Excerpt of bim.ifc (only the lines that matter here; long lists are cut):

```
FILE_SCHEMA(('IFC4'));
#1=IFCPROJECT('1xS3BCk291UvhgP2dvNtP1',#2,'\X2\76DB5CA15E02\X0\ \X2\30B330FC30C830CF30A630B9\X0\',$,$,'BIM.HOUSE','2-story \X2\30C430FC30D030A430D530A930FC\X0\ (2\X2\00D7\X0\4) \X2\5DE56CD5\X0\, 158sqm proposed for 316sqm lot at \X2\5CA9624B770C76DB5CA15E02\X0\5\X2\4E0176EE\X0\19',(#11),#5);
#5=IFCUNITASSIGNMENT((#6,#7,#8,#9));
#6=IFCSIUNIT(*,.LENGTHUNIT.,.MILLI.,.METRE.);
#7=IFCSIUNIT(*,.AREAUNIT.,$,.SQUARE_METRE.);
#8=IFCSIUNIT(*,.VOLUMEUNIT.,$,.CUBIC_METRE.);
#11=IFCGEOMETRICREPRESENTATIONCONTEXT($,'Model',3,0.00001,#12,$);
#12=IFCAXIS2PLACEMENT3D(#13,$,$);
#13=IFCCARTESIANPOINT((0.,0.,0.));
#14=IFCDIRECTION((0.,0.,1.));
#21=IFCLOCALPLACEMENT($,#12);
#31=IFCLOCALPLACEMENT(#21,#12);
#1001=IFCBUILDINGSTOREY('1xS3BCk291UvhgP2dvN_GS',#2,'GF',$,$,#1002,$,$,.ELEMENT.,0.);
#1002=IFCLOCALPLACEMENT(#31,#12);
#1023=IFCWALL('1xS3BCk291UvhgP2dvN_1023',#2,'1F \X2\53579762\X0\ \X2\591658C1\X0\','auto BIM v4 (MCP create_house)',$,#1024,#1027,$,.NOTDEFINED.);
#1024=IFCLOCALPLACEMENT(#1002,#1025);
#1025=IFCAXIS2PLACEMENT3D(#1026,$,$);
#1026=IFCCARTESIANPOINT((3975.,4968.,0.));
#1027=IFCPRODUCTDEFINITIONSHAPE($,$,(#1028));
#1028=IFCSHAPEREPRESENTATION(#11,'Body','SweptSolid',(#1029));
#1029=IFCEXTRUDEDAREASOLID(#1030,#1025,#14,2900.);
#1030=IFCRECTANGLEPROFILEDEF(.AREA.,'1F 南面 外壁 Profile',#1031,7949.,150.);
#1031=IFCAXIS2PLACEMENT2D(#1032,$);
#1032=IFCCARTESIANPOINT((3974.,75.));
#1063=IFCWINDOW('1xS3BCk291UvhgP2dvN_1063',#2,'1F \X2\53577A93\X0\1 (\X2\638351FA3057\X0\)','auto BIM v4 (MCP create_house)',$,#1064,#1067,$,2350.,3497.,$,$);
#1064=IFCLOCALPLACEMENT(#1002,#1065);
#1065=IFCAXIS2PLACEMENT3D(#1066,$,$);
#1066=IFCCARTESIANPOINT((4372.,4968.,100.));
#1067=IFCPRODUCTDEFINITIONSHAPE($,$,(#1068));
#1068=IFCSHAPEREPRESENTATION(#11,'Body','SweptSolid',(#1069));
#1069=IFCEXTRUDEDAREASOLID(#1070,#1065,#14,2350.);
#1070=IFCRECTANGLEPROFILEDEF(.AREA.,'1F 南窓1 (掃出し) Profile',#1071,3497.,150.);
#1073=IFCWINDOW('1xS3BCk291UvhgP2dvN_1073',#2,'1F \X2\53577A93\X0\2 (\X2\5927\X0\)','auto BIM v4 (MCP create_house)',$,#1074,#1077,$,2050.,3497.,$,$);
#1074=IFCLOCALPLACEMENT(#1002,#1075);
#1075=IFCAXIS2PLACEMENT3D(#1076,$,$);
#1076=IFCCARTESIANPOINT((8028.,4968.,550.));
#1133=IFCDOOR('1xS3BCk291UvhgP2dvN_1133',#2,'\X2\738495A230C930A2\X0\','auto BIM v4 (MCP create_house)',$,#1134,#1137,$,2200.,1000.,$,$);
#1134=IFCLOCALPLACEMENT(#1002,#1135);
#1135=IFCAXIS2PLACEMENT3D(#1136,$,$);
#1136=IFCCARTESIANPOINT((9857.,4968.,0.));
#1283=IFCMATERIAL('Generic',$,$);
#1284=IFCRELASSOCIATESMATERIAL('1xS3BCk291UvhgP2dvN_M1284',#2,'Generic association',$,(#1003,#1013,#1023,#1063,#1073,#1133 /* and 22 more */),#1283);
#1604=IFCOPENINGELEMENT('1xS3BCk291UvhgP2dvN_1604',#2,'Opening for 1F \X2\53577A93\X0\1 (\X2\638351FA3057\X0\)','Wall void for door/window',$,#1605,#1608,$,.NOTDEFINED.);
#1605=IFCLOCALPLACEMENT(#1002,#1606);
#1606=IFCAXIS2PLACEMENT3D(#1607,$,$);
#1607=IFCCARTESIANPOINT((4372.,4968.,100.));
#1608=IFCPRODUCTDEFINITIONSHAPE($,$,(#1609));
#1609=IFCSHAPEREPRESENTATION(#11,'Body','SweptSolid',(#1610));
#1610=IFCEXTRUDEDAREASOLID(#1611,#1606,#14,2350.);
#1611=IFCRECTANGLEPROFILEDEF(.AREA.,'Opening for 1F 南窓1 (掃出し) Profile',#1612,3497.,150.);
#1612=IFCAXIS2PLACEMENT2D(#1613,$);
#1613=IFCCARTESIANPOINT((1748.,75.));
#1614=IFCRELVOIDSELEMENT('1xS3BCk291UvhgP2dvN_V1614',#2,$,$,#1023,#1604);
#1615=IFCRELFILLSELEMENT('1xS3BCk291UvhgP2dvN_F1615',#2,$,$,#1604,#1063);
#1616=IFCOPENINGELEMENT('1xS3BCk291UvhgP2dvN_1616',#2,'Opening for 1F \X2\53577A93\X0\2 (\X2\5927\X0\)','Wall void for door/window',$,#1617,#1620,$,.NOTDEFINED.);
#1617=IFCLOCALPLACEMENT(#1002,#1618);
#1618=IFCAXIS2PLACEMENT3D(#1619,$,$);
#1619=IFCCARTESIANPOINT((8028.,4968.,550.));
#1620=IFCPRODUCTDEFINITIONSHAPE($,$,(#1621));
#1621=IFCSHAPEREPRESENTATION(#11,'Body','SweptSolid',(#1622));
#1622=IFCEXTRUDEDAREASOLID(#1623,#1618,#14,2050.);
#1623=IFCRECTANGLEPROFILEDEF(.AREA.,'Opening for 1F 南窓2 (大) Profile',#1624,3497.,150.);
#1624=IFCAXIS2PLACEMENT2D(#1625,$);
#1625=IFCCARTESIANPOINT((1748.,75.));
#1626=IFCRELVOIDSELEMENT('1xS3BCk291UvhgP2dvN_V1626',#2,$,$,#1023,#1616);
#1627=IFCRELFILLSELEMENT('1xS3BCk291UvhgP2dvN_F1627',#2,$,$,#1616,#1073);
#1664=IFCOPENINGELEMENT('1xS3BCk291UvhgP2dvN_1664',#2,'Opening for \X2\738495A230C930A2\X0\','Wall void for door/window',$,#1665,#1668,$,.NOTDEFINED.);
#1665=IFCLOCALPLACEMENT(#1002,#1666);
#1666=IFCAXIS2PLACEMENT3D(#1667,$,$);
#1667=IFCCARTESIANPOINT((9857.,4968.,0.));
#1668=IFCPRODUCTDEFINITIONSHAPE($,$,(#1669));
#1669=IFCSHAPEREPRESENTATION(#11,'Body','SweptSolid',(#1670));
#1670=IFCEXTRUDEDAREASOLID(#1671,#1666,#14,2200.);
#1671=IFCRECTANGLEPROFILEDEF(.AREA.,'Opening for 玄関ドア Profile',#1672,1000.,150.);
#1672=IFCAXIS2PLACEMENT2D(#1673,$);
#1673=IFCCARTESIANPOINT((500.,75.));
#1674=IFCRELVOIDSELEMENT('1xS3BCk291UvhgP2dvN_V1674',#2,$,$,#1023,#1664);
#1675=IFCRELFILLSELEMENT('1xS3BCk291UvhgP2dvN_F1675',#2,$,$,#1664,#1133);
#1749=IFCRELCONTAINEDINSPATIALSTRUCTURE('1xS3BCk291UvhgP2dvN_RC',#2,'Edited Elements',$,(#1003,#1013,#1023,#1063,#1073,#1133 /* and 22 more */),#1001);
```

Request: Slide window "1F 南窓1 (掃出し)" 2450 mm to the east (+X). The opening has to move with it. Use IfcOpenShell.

```python
import ifcopenshell
import ifcopenshell.api.geometry
import ifcopenshell.util.placement

model = ifcopenshell.open("bim.ifc")

window = model.by_id(1063)
opening = window.FillsVoids[0].RelatingOpeningElement
wall = opening.VoidsElements[0].RelatingBuildingElement

wall_matrix = ifcopenshell.util.placement.get_local_placement(wall.ObjectPlacement)
shift = wall_matrix[:3, 0] * 2450.0
before = ifcopenshell.util.placement.get_local_placement(window.ObjectPlacement)[:3, 3].copy()

# The window is not placed relative to its opening, so move both.
for product in (opening, window):
    matrix = ifcopenshell.util.placement.get_local_placement(product.ObjectPlacement)
    matrix[:3, 3] += shift
    ifcopenshell.api.geometry.edit_object_placement(model, product=product, matrix=matrix, is_si=False)

after = ifcopenshell.util.placement.get_local_placement(window.ObjectPlacement)[:3, 3]
print("window moved by", (after - before).round(3) + 0.0)

model.write("bim_v2.ifc")
```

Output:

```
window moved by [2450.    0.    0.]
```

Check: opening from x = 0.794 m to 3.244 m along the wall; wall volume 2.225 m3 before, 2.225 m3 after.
